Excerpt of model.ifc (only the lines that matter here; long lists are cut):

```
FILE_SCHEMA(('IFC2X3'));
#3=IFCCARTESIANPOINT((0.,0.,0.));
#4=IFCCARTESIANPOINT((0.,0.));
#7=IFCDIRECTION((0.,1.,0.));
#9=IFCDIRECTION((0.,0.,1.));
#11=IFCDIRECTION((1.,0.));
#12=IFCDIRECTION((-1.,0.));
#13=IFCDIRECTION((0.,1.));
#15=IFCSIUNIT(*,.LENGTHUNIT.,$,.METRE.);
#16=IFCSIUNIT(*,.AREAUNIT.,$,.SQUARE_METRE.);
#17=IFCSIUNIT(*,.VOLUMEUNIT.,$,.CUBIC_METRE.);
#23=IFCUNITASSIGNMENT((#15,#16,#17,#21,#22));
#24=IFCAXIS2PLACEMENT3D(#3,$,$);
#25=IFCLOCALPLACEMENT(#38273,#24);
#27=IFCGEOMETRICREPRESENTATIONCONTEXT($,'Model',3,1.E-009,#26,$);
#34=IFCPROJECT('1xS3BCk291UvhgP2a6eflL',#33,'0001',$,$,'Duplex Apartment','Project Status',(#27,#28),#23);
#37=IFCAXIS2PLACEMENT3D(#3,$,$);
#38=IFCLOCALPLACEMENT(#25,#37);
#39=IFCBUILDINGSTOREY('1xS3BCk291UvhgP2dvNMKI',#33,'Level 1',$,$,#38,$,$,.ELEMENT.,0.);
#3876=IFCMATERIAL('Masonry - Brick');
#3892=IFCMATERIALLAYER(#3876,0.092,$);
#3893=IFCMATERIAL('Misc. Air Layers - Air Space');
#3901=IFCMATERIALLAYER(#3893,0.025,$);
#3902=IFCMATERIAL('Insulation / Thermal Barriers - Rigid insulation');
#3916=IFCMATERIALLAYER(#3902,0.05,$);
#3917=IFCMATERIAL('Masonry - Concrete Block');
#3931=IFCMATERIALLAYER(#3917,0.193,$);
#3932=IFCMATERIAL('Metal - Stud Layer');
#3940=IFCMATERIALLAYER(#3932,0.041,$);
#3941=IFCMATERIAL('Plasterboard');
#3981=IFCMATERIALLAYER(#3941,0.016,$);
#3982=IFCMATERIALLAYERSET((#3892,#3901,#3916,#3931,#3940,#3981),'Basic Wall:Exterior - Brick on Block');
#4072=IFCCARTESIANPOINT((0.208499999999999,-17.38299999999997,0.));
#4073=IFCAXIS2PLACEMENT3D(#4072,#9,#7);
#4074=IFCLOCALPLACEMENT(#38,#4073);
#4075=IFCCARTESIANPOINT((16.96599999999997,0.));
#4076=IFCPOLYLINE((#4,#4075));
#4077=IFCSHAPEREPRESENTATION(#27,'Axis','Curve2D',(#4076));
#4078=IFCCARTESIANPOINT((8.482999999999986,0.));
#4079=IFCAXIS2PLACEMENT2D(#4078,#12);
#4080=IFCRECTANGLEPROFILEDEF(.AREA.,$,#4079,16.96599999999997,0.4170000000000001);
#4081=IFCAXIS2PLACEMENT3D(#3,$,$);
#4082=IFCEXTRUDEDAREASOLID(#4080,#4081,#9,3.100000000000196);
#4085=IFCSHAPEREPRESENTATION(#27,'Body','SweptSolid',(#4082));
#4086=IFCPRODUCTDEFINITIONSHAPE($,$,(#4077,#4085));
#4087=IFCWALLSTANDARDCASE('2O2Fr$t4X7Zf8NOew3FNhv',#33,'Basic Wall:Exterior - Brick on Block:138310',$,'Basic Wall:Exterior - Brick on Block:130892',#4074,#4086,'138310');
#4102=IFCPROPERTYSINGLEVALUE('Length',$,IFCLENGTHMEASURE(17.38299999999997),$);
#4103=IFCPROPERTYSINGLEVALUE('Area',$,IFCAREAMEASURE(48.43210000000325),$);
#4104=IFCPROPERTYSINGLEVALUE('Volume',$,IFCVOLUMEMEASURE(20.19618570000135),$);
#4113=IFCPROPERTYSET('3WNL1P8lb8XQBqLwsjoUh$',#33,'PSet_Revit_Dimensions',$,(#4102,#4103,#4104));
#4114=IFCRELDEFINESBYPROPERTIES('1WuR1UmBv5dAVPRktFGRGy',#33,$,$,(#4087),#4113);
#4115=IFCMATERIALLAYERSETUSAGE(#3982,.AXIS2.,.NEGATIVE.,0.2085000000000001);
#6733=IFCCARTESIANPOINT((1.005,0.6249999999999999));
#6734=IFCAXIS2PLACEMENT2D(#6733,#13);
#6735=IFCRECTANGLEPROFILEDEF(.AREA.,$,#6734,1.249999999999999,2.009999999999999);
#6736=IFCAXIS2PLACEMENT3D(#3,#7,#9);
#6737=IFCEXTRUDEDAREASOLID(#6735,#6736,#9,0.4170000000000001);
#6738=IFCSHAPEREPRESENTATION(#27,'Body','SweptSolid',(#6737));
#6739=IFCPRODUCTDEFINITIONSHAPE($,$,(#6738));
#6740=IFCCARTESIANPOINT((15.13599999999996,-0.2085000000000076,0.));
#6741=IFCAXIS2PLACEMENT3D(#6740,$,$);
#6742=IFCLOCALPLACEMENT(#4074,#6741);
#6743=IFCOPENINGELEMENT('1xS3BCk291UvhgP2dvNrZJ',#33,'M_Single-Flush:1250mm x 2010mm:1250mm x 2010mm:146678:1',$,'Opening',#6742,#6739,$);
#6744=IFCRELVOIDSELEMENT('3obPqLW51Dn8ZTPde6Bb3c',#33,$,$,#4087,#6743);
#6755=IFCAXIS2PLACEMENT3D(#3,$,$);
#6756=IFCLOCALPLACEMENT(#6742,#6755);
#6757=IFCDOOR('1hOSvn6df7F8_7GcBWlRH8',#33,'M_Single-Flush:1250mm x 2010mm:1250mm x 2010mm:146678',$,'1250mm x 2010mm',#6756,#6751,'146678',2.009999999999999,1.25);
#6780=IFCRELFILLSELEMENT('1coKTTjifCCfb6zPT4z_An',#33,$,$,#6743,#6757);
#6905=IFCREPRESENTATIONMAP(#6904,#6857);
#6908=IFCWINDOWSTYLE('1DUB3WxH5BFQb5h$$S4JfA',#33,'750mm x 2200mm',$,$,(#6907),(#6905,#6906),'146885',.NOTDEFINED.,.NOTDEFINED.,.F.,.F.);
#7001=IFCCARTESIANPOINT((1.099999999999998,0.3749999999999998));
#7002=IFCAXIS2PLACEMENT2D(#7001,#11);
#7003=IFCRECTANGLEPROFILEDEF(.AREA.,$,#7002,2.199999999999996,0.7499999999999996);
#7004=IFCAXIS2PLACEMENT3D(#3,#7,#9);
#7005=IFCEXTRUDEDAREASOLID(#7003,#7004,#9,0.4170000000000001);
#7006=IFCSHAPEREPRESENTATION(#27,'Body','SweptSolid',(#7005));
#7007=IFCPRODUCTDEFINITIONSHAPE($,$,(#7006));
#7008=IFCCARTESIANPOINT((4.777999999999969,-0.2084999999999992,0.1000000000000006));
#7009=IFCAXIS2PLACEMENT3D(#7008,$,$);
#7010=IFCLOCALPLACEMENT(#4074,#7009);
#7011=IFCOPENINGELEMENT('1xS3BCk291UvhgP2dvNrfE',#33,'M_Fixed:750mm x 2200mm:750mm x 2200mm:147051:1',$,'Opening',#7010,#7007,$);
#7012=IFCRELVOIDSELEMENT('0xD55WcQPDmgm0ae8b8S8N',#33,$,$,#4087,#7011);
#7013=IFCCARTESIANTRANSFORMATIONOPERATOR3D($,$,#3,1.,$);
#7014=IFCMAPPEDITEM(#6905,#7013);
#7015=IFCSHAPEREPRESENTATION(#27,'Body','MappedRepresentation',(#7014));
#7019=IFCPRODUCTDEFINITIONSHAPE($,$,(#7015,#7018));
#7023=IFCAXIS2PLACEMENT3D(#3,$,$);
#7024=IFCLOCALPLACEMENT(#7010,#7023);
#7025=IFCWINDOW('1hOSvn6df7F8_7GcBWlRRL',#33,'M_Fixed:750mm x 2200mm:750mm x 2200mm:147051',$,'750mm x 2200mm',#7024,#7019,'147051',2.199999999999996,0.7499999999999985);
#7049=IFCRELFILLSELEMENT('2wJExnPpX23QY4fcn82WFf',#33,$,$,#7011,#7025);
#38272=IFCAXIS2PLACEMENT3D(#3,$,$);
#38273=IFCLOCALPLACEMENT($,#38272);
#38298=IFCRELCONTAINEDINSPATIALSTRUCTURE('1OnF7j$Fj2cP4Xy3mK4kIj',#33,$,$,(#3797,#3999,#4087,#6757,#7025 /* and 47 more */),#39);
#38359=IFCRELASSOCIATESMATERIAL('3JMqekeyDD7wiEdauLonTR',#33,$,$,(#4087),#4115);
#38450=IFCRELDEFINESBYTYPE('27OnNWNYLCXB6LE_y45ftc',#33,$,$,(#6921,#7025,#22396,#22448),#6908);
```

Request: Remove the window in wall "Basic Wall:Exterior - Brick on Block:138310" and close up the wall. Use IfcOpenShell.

```python
import ifcopenshell
import ifcopenshell.api.feature
import ifcopenshell.api.pset
import ifcopenshell.api.root
import ifcopenshell.geom
import ifcopenshell.util.element
import ifcopenshell.util.shape
import ifcopenshell.util.unit

model = ifcopenshell.open("model.ifc")
area_scale = ifcopenshell.util.unit.calculate_unit_scale(model, "AREAUNIT")
volume_scale = ifcopenshell.util.unit.calculate_unit_scale(model, "VOLUMEUNIT")
settings = ifcopenshell.geom.settings()


def volume(element):
    """Net volume in cubic metres, openings subtracted."""
    shape = ifcopenshell.geom.create_shape(settings, element)
    return ifcopenshell.util.shape.get_volume(shape.geometry)


window = model.by_guid("1hOSvn6df7F8_7GcBWlRRL")
opening = window.FillsVoids[0].RelatingOpeningElement
wall = opening.VoidsElements[0].RelatingBuildingElement
before = volume(wall)

ifcopenshell.api.root.remove_product(model, product=window)
ifcopenshell.api.feature.remove_feature(model, feature=opening)

after = volume(wall)
thickness = 0.417  # wall thickness in metres

# Update the wall's stored quantities.
pset = model.by_id(ifcopenshell.util.element.get_pset(wall, "PSet_Revit_Dimensions", should_inherit=False)["id"])
ifcopenshell.api.pset.edit_pset(model, pset=pset, properties={
    "Area": model.create_entity("IfcAreaMeasure", after / thickness / area_scale),
    "Volume": model.create_entity("IfcVolumeMeasure", after / volume_scale),
})

print(f"wall volume {before:.3f} -> {after:.3f} m3")

model.write("model_edited.ifc")
```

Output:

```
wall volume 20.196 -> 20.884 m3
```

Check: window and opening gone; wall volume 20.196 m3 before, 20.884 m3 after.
